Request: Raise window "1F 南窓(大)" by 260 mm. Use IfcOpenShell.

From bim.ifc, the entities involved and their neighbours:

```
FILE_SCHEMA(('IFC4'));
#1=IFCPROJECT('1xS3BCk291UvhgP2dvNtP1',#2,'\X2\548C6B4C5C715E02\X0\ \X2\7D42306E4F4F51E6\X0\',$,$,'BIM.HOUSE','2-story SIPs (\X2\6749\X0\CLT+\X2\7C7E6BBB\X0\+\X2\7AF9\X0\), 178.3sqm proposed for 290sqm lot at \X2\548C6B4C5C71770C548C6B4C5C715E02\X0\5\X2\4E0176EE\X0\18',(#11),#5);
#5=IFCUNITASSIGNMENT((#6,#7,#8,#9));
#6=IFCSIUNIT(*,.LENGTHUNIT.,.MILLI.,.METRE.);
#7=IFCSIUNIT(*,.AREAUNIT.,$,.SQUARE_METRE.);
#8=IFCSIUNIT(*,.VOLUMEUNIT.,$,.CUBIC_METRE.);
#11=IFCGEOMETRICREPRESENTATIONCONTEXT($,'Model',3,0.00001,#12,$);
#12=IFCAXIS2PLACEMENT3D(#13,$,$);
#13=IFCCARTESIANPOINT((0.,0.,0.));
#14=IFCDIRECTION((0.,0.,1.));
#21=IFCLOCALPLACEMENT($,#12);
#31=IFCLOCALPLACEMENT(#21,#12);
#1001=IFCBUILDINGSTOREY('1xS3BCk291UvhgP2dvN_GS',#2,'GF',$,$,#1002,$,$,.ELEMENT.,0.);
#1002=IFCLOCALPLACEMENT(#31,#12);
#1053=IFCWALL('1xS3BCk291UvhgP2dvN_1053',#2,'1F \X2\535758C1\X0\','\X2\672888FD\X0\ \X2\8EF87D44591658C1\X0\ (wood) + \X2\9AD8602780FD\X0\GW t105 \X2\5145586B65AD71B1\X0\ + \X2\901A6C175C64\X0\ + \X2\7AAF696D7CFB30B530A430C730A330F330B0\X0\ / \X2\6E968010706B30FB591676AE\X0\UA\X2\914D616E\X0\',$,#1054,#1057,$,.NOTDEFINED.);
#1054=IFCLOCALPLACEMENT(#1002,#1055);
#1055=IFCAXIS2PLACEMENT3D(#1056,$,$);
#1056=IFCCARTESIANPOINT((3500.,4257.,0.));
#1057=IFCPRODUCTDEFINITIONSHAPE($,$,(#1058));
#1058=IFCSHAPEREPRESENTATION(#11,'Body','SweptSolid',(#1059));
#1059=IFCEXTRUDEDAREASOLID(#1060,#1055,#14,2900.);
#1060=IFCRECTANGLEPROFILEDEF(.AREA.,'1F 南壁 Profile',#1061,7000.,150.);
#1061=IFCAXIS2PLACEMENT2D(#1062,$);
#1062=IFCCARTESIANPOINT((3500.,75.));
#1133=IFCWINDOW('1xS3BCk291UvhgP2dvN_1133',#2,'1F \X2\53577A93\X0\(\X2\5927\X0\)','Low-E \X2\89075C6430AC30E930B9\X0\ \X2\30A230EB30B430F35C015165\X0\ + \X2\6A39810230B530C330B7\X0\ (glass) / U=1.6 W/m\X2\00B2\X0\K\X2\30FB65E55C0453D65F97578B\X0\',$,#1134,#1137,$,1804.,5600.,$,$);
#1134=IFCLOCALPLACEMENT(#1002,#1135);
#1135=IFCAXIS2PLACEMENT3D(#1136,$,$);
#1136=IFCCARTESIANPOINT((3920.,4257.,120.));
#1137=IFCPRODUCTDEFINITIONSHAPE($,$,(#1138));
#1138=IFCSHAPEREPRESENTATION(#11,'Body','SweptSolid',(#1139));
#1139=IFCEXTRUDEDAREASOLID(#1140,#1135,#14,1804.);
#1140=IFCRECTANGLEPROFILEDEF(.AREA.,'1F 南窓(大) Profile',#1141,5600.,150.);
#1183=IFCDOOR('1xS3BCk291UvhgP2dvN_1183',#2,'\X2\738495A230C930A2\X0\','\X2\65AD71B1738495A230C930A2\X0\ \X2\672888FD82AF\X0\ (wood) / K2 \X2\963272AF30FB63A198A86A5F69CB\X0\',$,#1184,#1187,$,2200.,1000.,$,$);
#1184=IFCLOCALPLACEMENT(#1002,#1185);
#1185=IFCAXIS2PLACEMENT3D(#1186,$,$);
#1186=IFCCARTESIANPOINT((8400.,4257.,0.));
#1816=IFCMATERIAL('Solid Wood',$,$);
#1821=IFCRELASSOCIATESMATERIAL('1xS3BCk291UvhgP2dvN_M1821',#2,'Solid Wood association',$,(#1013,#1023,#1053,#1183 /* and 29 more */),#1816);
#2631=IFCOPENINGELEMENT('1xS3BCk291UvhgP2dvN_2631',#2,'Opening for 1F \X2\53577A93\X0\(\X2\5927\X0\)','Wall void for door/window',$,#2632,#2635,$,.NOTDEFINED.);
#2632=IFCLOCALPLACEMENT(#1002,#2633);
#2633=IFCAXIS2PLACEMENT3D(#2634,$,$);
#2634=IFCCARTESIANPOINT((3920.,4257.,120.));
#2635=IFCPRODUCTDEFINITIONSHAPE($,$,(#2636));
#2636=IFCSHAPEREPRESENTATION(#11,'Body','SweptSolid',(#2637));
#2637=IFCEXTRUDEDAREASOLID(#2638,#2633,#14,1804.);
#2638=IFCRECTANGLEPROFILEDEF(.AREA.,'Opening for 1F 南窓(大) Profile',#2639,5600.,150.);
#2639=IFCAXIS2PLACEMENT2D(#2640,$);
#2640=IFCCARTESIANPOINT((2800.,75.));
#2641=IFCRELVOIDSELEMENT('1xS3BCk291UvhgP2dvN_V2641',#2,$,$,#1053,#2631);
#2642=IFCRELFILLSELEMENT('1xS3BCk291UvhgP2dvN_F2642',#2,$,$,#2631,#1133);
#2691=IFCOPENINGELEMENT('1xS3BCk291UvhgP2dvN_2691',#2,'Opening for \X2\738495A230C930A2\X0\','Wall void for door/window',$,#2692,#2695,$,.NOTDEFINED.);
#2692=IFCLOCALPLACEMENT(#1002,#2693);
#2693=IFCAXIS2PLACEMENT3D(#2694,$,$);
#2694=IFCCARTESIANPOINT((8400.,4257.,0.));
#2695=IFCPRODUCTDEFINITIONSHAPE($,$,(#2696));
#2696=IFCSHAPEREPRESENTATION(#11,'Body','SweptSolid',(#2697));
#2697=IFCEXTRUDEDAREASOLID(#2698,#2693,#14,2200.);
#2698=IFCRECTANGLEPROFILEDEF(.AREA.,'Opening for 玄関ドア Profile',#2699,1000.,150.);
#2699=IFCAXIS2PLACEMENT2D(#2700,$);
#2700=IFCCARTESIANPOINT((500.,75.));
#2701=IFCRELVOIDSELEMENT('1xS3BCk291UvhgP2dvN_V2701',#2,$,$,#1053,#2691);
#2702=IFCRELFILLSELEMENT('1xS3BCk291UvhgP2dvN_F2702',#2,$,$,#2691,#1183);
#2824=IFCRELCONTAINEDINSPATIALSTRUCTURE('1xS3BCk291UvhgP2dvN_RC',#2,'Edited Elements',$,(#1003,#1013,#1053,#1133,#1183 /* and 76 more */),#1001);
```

```python
import numpy as np
import ifcopenshell
import ifcopenshell.api.geometry
import ifcopenshell.util.placement
import ifcopenshell.util.unit

model = ifcopenshell.open("bim.ifc")
unit_scale = ifcopenshell.util.unit.calculate_unit_scale(model)

window = model.by_guid("1xS3BCk291UvhgP2dvN_1133")
opening = window.FillsVoids[0].RelatingOpeningElement
dz = 260.0

shift = np.array([0.0, 0.0, dz])
# The window is not placed relative to its opening, so move both.
for product in (opening, window):
    matrix = ifcopenshell.util.placement.get_local_placement(product.ObjectPlacement)
    matrix[:3, 3] += shift
    ifcopenshell.api.geometry.edit_object_placement(model, product=product, matrix=matrix, is_si=False)

print(f"moved by {dz * unit_scale:+.3f} m")

model.write("bim_rev.ifc")
```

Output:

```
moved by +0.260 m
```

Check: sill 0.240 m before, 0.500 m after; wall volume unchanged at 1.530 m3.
